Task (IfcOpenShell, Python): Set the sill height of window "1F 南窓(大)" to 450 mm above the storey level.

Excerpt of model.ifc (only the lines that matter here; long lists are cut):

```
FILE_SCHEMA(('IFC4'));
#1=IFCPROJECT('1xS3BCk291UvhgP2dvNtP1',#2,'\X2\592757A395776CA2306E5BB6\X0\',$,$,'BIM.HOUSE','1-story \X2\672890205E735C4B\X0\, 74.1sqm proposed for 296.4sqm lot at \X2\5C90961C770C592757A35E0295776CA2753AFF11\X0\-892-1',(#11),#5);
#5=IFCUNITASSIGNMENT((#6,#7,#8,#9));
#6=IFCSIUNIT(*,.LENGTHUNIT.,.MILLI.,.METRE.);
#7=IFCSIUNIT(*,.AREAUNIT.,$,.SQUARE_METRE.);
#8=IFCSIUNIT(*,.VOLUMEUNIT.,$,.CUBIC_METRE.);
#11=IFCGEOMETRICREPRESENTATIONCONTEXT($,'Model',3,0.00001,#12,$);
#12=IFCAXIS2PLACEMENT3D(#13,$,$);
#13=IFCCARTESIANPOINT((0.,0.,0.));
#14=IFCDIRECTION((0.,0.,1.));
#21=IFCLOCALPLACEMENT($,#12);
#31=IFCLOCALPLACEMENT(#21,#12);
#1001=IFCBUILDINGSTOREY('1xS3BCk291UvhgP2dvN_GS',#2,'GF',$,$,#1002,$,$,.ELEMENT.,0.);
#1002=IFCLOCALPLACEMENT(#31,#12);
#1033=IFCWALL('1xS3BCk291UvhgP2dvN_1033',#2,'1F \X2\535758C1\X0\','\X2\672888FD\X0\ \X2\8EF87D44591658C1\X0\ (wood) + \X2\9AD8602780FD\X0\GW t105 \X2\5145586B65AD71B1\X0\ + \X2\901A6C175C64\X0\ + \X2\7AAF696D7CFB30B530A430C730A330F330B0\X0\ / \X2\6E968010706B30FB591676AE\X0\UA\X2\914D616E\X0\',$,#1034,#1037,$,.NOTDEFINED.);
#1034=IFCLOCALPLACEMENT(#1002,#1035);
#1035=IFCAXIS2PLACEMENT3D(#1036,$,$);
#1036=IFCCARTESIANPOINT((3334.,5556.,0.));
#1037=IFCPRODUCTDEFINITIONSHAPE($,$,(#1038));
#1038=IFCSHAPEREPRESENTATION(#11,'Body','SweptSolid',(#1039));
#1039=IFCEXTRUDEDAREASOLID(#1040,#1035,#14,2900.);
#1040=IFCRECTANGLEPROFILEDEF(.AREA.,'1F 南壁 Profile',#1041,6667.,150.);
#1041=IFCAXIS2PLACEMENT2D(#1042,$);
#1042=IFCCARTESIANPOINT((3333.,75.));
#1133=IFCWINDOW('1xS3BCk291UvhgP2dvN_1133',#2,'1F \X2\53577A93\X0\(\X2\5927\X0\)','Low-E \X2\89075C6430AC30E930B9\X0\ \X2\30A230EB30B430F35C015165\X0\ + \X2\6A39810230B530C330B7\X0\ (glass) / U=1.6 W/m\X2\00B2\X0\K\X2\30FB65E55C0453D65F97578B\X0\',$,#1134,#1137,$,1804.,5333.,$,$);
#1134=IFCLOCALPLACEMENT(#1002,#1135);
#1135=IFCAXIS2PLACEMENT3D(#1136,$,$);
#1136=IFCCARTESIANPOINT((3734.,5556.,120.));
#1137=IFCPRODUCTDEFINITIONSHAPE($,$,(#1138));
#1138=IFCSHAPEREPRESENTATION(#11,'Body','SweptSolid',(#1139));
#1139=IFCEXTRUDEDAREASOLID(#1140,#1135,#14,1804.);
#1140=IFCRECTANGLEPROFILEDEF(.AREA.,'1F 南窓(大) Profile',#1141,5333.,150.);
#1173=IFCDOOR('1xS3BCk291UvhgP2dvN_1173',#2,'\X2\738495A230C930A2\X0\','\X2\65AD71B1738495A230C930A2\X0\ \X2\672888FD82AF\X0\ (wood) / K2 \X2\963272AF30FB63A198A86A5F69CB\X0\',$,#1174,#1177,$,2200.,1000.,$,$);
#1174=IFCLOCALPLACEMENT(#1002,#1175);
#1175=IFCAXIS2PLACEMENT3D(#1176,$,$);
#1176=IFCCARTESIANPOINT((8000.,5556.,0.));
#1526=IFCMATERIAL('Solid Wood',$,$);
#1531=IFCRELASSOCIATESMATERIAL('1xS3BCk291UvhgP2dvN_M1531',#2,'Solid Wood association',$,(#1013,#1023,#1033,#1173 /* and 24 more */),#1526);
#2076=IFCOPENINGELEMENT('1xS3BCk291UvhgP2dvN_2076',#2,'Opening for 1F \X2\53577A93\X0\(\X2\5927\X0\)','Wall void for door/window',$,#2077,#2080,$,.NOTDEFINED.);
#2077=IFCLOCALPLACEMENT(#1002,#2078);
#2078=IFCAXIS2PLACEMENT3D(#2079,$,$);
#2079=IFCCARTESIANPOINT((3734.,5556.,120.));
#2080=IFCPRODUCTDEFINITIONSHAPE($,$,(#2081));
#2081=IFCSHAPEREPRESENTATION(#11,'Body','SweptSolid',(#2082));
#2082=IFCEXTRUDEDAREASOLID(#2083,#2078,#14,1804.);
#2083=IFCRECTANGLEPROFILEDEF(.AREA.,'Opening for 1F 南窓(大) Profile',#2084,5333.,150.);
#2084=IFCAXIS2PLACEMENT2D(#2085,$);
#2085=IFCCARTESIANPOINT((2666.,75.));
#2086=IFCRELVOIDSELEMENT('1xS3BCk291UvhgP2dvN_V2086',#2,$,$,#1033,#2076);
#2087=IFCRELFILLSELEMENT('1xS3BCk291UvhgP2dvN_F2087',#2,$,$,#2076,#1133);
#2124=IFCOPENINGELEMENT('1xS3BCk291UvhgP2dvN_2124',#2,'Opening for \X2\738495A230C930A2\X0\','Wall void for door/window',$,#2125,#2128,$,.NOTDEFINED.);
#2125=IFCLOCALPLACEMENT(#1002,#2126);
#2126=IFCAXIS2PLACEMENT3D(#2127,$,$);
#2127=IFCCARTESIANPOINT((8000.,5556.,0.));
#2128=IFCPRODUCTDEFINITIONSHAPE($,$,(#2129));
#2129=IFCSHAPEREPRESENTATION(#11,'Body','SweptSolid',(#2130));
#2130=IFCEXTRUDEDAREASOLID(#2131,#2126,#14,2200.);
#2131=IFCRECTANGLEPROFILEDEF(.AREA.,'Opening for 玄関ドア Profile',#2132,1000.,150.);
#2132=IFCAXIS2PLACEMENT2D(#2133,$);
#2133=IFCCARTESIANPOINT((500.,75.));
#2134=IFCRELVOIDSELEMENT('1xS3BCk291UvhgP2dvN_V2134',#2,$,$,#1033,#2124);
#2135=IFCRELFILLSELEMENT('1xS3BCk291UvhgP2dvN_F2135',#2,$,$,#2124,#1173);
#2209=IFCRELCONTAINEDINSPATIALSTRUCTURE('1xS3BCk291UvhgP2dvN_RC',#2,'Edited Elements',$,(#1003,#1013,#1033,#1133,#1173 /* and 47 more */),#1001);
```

```python
import numpy as np
import ifcopenshell
import ifcopenshell.api.geometry
import ifcopenshell.geom
import ifcopenshell.util.element
import ifcopenshell.util.placement
import ifcopenshell.util.shape
import ifcopenshell.util.unit

model = ifcopenshell.open("model.ifc")
unit_scale = ifcopenshell.util.unit.calculate_unit_scale(model)

window = model.by_id(1133)
opening = window.FillsVoids[0].RelatingOpeningElement
storey = ifcopenshell.util.element.get_container(window, ifc_class="IfcBuildingStorey")
level = ifcopenshell.util.placement.get_local_placement(storey.ObjectPlacement)[2, 3]

# The opening's origin need not be at the sill, so measure its lowest point.
shape = ifcopenshell.geom.create_shape(ifcopenshell.geom.settings(), opening)
bottom = ifcopenshell.util.shape.get_shape_bottom_elevation(shape, shape.geometry) / unit_scale
dz = level + 450.0 - bottom

shift = np.array([0.0, 0.0, dz])
# The window is not placed relative to its opening, so move both.
for product in (opening, window):
    matrix = ifcopenshell.util.placement.get_local_placement(product.ObjectPlacement)
    matrix[:3, 3] += shift
    ifcopenshell.api.geometry.edit_object_placement(model, product=product, matrix=matrix, is_si=False)

print(f"moved by {dz * unit_scale:+.3f} m")

model.write("model_edited.ifc")
```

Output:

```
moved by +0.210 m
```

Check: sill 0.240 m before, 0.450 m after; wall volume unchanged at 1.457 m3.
